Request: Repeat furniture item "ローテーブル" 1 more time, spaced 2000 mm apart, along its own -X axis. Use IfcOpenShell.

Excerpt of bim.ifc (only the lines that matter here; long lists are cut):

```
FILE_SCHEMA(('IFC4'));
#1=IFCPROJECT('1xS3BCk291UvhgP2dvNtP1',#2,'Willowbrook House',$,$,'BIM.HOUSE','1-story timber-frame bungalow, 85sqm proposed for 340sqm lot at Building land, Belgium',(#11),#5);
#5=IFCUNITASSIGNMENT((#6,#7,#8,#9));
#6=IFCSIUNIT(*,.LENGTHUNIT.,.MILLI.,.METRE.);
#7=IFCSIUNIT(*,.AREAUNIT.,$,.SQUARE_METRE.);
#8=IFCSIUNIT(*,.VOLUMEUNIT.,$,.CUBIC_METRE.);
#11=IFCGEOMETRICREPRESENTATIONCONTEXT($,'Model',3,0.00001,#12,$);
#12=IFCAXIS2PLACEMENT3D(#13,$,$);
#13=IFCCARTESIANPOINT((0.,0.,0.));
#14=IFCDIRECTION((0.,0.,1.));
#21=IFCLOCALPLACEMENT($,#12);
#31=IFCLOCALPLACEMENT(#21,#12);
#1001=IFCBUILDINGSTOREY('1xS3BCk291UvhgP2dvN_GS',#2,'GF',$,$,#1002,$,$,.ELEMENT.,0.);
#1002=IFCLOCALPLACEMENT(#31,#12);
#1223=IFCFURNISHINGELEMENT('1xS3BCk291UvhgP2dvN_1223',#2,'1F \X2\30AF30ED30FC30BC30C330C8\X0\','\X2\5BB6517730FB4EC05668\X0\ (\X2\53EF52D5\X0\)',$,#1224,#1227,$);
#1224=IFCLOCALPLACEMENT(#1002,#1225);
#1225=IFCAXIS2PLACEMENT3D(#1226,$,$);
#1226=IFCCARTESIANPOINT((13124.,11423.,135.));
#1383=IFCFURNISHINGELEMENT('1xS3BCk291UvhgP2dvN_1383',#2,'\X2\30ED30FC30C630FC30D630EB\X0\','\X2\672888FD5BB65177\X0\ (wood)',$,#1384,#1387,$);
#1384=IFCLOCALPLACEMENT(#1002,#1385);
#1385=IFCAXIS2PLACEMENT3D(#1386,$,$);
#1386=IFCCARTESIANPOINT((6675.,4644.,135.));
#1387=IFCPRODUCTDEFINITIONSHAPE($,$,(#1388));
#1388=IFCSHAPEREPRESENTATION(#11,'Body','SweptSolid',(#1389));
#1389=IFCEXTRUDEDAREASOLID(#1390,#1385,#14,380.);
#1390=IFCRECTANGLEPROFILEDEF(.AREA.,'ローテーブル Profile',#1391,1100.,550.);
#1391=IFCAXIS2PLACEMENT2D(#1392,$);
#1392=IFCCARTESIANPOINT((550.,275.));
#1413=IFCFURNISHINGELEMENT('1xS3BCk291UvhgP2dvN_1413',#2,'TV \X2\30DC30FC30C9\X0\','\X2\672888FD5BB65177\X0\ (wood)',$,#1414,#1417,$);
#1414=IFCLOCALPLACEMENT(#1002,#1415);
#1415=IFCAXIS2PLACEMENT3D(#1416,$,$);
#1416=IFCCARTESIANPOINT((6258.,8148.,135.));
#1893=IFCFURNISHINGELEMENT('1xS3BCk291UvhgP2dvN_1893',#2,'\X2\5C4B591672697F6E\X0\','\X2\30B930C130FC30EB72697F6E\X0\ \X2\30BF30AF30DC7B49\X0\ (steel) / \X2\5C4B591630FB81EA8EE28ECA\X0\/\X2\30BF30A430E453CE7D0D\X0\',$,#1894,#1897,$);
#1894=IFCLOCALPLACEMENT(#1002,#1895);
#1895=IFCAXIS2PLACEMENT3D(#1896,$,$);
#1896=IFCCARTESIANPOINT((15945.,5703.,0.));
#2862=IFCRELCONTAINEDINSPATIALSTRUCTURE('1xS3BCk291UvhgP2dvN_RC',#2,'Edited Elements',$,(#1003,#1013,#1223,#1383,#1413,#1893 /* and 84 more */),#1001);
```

```python
import ifcopenshell
import ifcopenshell.api.geometry
import ifcopenshell.api.root
import ifcopenshell.util.element
import ifcopenshell.util.placement
import ifcopenshell.util.unit

model = ifcopenshell.open("bim.ifc")
unit_scale = ifcopenshell.util.unit.calculate_unit_scale(model)


def reuse_history(source, copy):
    """copy_class also copies each property set's owner history, people and application; keep the originals."""
    for rel in copy.IsDefinedBy:
        if rel.is_a("IfcRelDefinesByProperties") and (history := rel.RelatingPropertyDefinition.OwnerHistory):
            rel.RelatingPropertyDefinition.OwnerHistory = source.OwnerHistory
            ifcopenshell.util.element.remove_deep2(model, history)


source = model.by_id(1383)
base = ifcopenshell.util.placement.get_local_placement(source.ObjectPlacement)
step = -base[:3, 0] * 2 / unit_scale

for i in range(1, 2):
    copy = ifcopenshell.api.root.copy_class(model, product=source)
    copy.Representation = ifcopenshell.util.element.copy_deep(
        model, source.Representation, exclude=["IfcGeometricRepresentationContext", "IfcRepresentationMap"]
    )
    reuse_history(source, copy)
    matrix = base.copy()
    matrix[:3, 3] += i * step
    print("added at", matrix[:3, 3].round(3) + 0.0)
    ifcopenshell.api.geometry.edit_object_placement(model, product=copy, matrix=matrix, is_si=False)

model.write("bim-out.ifc")
```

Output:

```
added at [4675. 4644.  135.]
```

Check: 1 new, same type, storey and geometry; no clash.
